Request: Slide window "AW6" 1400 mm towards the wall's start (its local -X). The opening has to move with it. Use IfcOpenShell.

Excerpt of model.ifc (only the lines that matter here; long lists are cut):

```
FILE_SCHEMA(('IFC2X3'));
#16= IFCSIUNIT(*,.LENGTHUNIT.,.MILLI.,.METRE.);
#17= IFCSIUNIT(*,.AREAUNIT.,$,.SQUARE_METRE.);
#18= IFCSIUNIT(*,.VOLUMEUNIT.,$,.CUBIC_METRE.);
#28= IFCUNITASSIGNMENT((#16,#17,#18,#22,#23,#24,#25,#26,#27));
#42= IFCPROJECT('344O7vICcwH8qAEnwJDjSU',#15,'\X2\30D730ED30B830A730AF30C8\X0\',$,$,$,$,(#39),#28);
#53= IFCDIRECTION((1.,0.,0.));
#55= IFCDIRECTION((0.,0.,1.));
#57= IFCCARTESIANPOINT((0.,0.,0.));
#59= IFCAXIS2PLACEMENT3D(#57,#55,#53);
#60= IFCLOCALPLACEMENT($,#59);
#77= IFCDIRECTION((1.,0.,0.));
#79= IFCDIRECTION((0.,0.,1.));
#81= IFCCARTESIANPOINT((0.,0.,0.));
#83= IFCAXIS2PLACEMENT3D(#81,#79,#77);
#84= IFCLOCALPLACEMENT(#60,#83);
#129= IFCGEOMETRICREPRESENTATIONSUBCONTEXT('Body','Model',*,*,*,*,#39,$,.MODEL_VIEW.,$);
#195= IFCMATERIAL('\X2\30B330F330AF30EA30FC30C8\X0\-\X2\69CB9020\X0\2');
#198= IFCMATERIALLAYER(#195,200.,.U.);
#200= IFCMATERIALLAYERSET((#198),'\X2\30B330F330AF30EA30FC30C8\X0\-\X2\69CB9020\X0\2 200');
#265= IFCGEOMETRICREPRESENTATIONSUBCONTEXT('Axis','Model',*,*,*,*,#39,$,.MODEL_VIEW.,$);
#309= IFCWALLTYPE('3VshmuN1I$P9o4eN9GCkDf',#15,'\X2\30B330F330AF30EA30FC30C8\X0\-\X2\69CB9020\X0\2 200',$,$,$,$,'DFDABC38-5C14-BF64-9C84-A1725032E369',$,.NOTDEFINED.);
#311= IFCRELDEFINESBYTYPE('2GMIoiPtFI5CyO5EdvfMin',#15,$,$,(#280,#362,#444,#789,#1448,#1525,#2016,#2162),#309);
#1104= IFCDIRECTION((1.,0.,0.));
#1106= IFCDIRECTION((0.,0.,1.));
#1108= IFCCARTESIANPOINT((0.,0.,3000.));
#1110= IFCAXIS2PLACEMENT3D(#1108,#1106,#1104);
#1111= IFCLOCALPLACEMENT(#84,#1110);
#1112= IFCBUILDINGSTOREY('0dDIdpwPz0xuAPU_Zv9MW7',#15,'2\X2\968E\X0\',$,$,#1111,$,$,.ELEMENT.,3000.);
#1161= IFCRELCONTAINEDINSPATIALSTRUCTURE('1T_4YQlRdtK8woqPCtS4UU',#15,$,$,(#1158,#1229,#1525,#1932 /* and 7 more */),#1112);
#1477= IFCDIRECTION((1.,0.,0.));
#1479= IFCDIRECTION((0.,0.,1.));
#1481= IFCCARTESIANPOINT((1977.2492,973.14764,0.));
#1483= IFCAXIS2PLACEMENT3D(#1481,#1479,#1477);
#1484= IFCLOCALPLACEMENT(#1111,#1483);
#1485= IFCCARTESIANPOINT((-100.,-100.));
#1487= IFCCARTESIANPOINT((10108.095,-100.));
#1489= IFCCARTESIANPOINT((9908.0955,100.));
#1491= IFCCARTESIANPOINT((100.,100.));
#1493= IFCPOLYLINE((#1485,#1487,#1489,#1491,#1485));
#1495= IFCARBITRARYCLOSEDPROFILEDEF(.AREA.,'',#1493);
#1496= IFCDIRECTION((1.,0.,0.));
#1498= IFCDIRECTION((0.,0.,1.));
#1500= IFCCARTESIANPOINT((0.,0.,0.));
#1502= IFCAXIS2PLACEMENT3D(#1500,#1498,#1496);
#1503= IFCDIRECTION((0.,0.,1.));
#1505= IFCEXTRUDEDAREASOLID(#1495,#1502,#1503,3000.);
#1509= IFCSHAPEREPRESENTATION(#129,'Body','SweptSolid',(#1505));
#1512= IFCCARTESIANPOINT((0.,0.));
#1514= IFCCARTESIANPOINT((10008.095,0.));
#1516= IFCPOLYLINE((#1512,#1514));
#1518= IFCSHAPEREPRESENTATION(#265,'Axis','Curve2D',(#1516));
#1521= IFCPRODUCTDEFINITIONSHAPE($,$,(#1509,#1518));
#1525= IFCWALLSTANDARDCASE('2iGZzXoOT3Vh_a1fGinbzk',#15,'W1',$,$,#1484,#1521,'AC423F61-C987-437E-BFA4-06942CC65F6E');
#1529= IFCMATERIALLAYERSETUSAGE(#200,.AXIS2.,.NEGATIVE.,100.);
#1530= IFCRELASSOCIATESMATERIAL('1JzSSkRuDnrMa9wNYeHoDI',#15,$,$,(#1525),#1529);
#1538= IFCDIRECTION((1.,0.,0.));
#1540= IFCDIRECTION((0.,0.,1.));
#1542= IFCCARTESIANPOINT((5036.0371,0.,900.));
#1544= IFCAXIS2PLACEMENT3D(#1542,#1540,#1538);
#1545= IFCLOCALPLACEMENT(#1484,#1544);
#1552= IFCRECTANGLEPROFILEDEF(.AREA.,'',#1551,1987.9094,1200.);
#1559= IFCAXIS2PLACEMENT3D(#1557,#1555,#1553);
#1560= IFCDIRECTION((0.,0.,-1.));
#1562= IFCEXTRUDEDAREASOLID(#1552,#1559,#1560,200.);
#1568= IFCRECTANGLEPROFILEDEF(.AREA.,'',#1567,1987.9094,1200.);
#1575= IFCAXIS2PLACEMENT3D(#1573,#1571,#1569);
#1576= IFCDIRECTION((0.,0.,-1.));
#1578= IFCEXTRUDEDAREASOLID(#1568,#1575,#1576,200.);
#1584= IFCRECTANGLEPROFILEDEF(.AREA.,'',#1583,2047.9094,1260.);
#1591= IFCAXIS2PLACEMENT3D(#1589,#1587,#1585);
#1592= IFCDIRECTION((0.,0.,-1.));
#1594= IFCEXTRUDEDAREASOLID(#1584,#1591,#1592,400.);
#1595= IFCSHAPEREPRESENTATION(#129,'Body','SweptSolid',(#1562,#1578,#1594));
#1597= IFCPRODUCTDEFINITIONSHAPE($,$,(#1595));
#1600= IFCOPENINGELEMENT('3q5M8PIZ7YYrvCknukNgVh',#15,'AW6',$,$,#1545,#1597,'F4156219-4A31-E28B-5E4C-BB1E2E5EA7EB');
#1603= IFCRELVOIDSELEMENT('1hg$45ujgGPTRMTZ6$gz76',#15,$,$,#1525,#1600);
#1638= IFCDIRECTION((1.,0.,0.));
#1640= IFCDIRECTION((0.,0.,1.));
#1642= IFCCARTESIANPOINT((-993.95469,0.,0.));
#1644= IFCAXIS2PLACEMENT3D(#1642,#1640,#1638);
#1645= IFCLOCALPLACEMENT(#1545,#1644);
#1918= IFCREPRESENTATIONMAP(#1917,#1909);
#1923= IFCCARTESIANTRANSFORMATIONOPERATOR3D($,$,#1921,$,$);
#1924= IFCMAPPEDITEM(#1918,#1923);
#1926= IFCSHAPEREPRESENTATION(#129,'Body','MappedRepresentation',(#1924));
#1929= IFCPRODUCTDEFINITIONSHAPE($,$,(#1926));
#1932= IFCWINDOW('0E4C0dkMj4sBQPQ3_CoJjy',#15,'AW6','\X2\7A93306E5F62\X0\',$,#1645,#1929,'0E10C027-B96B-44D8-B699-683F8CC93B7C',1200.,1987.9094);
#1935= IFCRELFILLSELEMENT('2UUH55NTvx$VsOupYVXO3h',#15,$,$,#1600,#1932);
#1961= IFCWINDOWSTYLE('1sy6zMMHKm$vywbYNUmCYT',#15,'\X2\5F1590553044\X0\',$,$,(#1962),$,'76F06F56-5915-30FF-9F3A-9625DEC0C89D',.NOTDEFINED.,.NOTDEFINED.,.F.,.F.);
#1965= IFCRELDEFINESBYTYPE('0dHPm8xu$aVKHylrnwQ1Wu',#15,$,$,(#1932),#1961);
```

```python
import ifcopenshell
import ifcopenshell.api.geometry
import ifcopenshell.util.placement
import ifcopenshell.util.unit

model = ifcopenshell.open("model.ifc")
unit_scale = ifcopenshell.util.unit.calculate_unit_scale(model)

window = model.by_guid("0E4C0dkMj4sBQPQ3_CoJjy")
opening = window.FillsVoids[0].RelatingOpeningElement
wall = opening.VoidsElements[0].RelatingBuildingElement

wall_matrix = ifcopenshell.util.placement.get_local_placement(wall.ObjectPlacement)
shift = wall_matrix[:3, 0] * -1.4 / unit_scale
before = ifcopenshell.util.placement.get_local_placement(window.ObjectPlacement)[:3, 3].copy()

# The window is placed relative to its opening, so it follows when the opening moves.
matrix = ifcopenshell.util.placement.get_local_placement(opening.ObjectPlacement)
matrix[:3, 3] += shift
ifcopenshell.api.geometry.edit_object_placement(
    model, product=opening, matrix=matrix, is_si=False, should_transform_children=True
)

after = ifcopenshell.util.placement.get_local_placement(window.ObjectPlacement)[:3, 3]
print("window moved by", (after - before).round(3) + 0.0)

model.write("model_rev.ifc")
```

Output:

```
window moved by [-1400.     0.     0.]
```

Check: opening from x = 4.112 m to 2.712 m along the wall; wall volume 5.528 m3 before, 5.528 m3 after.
